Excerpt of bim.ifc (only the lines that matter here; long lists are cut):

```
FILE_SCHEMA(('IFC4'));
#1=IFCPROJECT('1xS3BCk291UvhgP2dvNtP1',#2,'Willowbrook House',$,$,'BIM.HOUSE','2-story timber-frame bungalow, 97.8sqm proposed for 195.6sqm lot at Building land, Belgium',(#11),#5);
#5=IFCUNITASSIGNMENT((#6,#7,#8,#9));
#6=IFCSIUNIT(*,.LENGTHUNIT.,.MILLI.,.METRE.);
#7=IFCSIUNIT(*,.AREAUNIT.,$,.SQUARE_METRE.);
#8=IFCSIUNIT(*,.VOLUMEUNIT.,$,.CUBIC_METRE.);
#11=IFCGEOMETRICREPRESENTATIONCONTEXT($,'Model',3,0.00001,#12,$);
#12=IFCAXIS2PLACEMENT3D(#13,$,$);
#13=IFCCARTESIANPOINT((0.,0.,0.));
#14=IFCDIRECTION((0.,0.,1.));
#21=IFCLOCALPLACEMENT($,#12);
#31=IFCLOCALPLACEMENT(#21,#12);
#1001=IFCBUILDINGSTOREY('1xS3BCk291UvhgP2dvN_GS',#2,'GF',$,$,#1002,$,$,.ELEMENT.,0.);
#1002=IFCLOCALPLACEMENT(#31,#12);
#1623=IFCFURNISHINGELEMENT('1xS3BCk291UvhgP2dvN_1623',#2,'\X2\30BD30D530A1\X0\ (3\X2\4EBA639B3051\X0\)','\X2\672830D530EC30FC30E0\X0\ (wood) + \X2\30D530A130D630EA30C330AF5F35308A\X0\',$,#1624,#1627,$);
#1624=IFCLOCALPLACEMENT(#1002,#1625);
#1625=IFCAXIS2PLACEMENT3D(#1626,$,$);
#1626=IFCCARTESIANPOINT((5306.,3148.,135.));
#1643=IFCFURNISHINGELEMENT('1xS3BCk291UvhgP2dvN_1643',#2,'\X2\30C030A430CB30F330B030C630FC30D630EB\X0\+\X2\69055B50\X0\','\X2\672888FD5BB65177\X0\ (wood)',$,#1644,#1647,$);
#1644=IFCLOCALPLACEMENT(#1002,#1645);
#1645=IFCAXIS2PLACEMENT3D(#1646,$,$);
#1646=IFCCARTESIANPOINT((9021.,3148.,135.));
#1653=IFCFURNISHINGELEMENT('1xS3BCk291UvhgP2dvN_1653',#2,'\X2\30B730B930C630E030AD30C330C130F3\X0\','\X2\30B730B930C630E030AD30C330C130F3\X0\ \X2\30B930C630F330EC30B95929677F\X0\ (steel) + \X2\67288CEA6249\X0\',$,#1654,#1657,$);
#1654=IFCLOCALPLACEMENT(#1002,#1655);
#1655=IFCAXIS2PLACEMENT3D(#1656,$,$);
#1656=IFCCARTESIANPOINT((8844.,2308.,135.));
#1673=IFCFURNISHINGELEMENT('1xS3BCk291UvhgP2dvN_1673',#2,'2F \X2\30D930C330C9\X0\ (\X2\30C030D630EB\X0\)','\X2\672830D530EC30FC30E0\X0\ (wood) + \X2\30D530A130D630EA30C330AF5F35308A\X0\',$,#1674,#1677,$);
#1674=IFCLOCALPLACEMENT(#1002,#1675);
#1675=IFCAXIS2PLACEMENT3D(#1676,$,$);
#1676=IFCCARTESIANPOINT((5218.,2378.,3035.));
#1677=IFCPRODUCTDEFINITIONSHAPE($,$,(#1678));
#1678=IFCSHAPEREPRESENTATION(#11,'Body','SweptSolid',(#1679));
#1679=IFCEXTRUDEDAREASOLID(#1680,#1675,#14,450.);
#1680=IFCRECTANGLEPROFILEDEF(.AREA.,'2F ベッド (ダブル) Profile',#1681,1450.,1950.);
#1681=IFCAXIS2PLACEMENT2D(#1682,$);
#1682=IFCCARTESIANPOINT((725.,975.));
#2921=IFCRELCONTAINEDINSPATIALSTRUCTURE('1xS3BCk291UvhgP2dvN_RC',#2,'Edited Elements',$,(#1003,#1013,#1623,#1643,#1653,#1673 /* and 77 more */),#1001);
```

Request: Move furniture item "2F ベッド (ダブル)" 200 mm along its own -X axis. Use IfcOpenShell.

```python
import ifcopenshell
import ifcopenshell.api.geometry
import ifcopenshell.util.placement

model = ifcopenshell.open("bim.ifc")

item = model.by_guid("1xS3BCk291UvhgP2dvN_1673")
matrix = ifcopenshell.util.placement.get_local_placement(item.ObjectPlacement)
matrix[:3, 3] -= matrix[:3, 0] * 200.0
ifcopenshell.api.geometry.edit_object_placement(model, product=item, matrix=matrix, is_si=False)

print(ifcopenshell.util.placement.get_local_placement(item.ObjectPlacement).round(3) + 0.0)

model.write("bim_updated.ifc")
```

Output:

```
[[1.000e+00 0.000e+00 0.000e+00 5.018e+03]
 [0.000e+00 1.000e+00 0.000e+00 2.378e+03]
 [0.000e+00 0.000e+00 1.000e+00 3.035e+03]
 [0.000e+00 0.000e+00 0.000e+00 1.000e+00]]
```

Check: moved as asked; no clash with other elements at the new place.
